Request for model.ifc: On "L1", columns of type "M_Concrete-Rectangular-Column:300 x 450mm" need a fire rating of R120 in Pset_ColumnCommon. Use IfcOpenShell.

First a look at what the model holds.

```python
import ifcopenshell
import ifcopenshell.util.element

model = ifcopenshell.open("model.ifc")
print(model.schema)
storey = next(s for s in model.by_type("IfcBuildingStorey") if s.Name == "L1")
columns = [e for e in ifcopenshell.util.element.get_decomposition(storey) if e.is_a("IfcColumn")]
seen = {}
for e in columns:
    element_type = ifcopenshell.util.element.get_type(e)
    key = (element_type.Name if element_type != e and element_type else None, ifcopenshell.util.element.get_pset(e, "Pset_ColumnCommon", "FireRating"))
    seen[key] = seen.get(key, 0) + 1
for (name, value), count in sorted(seen.items(), key=str):
    print(count, "x", name, "|", value)
```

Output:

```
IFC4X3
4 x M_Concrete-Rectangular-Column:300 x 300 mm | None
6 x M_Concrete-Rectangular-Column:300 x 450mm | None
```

```python
import ifcopenshell
import ifcopenshell.api.pset
import ifcopenshell.util.element

model = ifcopenshell.open("model.ifc")

storey = next(s for s in model.by_type("IfcBuildingStorey") if s.Name == "L1")
columns = [e for e in ifcopenshell.util.element.get_decomposition(storey) if e.is_a("IfcColumn")]

count = 0
for e in columns:
    element_type = ifcopenshell.util.element.get_type(e)
    if element_type in (None, e) or element_type.Name != "M_Concrete-Rectangular-Column:300 x 450mm":
        continue
    # add_pset returns the element's existing set when there is one.
    pset = ifcopenshell.api.pset.add_pset(model, product=e, name="Pset_ColumnCommon")
    ifcopenshell.api.pset.edit_pset(model, pset=pset, properties={"FireRating": "R120"})
    count += 1

print(count, "columns updated")

model.write("model-out.ifc")
```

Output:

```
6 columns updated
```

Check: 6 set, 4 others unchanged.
